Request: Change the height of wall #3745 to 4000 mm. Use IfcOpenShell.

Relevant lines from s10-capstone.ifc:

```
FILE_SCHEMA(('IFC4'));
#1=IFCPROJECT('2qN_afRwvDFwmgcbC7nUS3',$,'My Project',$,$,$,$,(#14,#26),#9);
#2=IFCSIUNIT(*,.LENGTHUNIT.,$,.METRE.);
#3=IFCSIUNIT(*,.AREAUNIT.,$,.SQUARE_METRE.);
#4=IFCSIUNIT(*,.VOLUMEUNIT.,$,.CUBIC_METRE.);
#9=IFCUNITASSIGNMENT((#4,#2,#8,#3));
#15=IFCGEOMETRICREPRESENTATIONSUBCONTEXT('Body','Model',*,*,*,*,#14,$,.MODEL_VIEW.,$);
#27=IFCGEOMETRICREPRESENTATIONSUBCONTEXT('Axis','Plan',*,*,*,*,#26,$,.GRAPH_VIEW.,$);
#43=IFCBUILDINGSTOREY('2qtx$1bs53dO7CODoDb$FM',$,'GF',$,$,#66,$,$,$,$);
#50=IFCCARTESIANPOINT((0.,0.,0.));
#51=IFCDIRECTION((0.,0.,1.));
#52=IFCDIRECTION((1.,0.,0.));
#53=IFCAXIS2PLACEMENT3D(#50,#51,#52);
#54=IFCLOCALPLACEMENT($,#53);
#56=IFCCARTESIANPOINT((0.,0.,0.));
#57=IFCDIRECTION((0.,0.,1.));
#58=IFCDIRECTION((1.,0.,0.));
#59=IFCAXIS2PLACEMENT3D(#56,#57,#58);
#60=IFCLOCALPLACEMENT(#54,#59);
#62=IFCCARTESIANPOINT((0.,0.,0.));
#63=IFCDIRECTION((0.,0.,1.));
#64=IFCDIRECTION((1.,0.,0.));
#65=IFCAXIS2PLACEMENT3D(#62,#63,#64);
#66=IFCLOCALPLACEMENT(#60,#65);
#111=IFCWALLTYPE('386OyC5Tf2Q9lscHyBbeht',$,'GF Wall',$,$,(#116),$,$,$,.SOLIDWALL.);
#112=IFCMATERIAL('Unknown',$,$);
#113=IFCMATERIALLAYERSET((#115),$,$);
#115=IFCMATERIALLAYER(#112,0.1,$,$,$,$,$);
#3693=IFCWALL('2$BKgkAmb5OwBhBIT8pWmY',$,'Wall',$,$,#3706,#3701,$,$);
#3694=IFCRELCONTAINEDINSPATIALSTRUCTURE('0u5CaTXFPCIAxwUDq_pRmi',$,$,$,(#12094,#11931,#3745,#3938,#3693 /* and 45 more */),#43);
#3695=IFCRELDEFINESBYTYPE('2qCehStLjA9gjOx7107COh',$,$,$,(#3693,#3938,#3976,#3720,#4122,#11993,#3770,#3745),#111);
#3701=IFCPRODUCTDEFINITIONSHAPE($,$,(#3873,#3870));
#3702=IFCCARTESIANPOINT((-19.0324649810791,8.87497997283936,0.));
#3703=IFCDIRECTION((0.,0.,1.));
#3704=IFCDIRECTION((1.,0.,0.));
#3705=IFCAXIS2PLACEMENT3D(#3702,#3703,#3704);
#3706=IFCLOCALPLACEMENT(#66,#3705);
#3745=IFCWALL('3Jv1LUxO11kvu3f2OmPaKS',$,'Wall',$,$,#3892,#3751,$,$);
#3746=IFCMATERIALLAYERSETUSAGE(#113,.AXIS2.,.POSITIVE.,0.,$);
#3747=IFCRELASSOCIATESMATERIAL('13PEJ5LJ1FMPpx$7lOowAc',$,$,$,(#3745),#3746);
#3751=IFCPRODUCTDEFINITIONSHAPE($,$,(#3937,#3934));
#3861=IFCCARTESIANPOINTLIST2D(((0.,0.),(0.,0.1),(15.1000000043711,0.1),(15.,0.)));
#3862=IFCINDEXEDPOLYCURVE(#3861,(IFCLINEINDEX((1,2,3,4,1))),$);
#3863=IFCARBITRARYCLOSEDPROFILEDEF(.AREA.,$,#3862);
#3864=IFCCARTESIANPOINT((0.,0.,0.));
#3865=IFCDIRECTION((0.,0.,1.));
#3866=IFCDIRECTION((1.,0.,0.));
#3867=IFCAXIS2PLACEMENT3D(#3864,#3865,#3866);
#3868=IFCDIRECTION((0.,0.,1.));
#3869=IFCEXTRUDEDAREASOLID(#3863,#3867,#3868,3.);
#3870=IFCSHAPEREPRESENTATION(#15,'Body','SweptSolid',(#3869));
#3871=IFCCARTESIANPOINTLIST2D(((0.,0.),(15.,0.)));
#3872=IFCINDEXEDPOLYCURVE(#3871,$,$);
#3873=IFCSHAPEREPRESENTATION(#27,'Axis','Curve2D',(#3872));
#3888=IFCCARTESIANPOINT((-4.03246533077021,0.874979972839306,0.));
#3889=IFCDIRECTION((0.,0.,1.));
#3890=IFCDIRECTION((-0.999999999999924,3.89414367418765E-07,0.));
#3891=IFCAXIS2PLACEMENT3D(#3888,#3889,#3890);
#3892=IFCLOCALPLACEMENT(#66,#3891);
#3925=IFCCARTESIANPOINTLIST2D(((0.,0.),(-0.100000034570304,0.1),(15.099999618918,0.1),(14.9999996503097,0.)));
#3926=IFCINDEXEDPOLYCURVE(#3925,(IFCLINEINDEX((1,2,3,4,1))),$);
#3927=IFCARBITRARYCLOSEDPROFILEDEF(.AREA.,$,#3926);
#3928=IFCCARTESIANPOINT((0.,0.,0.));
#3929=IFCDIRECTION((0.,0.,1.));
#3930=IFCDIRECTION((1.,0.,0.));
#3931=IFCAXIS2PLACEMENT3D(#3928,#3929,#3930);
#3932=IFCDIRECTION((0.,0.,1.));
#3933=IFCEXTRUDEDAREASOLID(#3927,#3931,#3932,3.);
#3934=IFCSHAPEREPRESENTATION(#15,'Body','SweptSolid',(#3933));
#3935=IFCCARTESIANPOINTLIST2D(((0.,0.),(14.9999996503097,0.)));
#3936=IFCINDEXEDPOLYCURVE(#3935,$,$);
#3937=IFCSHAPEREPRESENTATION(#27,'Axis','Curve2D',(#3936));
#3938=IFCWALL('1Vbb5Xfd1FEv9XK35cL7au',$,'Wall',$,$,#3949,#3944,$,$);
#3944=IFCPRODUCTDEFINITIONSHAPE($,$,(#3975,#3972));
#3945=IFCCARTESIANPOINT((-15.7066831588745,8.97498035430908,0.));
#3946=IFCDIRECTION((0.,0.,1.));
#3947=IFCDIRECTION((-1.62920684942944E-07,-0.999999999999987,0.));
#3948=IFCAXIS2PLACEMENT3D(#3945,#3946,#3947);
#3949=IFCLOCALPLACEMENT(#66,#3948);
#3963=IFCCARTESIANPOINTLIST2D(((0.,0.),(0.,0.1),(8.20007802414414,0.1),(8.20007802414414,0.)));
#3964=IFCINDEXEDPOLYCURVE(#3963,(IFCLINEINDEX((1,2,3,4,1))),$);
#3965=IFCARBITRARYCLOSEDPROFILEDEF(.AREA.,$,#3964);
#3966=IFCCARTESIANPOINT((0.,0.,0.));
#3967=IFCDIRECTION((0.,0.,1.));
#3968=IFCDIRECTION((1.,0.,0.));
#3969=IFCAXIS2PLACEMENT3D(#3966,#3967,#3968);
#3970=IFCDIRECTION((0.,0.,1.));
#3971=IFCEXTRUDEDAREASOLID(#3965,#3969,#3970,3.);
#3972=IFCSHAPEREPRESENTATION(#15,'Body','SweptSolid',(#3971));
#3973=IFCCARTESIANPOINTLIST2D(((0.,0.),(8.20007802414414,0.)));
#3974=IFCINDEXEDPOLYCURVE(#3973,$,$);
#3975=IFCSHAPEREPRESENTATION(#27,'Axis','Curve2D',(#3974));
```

```python
import ifcopenshell
import ifcopenshell.geom
import ifcopenshell.util.representation
import ifcopenshell.util.shape

model = ifcopenshell.open("s10-capstone.ifc")
settings = ifcopenshell.geom.settings()


def volume(element):
    """Net volume in cubic metres, openings subtracted."""
    shape = ifcopenshell.geom.create_shape(settings, element)
    return ifcopenshell.util.shape.get_volume(shape.geometry)


wall = model.by_guid("3Jv1LUxO11kvu3f2OmPaKS")
before = volume(wall)

body = ifcopenshell.util.representation.get_representation(wall, "Model", "Body")
solid = body.Items[0]
old_height = solid.Depth
solid.Depth = 4.0
after = volume(wall)

print(f"height {old_height:g} -> {solid.Depth:g}, volume {before:.3f} -> {after:.3f} m3")

model.write("s10-capstone_updated.ifc")
```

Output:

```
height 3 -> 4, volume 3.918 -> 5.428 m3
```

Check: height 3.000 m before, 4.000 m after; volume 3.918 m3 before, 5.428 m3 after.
